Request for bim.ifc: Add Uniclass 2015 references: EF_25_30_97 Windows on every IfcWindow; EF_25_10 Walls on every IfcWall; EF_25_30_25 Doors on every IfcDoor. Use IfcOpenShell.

First a look at what the model holds.

```python
import ifcopenshell

model = ifcopenshell.open("bim.ifc")
print(model.schema)
print("classifications:", [c.Name for c in model.by_type("IfcClassification")])
for ifc_class in ("IfcDoor", "IfcRoof", "IfcStair", "IfcWall", "IfcWindow"):
    print(ifc_class, len(model.by_type(ifc_class)))
```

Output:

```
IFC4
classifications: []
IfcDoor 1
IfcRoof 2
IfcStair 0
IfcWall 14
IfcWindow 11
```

```python
import ifcopenshell
import ifcopenshell.api.classification

model = ifcopenshell.open("bim.ifc")

system = ifcopenshell.api.classification.add_classification(model, classification="Uniclass 2015")

codes = {
    "IfcWindow": ("EF_25_30_97", "Windows"),
    "IfcWall": ("EF_25_10", "Walls"),
    "IfcDoor": ("EF_25_30_25", "Doors"),
}
for ifc_class, (code, name) in codes.items():
    products = model.by_type(ifc_class)
    ifcopenshell.api.classification.add_reference(
        model, products=products, classification=system, identification=code, name=name
    )
    print(code, len(products))

model.write("bim_edited.ifc")
```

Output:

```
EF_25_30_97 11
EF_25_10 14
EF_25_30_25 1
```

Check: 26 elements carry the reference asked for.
